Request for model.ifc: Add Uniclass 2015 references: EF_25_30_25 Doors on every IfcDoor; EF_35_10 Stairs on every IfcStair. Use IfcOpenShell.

First a look at what the model holds.

```python
import ifcopenshell

model = ifcopenshell.open("model.ifc")
print(model.schema)
print("classifications:", [c.Name for c in model.by_type("IfcClassification")])
for ifc_class in ("IfcDoor", "IfcRoof", "IfcStair", "IfcWall", "IfcWindow"):
    print(ifc_class, len(model.by_type(ifc_class)))
```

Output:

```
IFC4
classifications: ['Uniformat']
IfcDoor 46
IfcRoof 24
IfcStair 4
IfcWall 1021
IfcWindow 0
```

```python
import ifcopenshell
import ifcopenshell.api.classification

model = ifcopenshell.open("model.ifc")

system = ifcopenshell.api.classification.add_classification(model, classification="Uniclass 2015")

codes = {
    "IfcDoor": ("EF_25_30_25", "Doors"),
    "IfcStair": ("EF_35_10", "Stairs"),
}
for ifc_class, (code, name) in codes.items():
    products = model.by_type(ifc_class)
    ifcopenshell.api.classification.add_reference(
        model, products=products, classification=system, identification=code, name=name
    )
    print(code, len(products))

model.write("model_v2.ifc")
```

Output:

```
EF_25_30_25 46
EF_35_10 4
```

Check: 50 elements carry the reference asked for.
